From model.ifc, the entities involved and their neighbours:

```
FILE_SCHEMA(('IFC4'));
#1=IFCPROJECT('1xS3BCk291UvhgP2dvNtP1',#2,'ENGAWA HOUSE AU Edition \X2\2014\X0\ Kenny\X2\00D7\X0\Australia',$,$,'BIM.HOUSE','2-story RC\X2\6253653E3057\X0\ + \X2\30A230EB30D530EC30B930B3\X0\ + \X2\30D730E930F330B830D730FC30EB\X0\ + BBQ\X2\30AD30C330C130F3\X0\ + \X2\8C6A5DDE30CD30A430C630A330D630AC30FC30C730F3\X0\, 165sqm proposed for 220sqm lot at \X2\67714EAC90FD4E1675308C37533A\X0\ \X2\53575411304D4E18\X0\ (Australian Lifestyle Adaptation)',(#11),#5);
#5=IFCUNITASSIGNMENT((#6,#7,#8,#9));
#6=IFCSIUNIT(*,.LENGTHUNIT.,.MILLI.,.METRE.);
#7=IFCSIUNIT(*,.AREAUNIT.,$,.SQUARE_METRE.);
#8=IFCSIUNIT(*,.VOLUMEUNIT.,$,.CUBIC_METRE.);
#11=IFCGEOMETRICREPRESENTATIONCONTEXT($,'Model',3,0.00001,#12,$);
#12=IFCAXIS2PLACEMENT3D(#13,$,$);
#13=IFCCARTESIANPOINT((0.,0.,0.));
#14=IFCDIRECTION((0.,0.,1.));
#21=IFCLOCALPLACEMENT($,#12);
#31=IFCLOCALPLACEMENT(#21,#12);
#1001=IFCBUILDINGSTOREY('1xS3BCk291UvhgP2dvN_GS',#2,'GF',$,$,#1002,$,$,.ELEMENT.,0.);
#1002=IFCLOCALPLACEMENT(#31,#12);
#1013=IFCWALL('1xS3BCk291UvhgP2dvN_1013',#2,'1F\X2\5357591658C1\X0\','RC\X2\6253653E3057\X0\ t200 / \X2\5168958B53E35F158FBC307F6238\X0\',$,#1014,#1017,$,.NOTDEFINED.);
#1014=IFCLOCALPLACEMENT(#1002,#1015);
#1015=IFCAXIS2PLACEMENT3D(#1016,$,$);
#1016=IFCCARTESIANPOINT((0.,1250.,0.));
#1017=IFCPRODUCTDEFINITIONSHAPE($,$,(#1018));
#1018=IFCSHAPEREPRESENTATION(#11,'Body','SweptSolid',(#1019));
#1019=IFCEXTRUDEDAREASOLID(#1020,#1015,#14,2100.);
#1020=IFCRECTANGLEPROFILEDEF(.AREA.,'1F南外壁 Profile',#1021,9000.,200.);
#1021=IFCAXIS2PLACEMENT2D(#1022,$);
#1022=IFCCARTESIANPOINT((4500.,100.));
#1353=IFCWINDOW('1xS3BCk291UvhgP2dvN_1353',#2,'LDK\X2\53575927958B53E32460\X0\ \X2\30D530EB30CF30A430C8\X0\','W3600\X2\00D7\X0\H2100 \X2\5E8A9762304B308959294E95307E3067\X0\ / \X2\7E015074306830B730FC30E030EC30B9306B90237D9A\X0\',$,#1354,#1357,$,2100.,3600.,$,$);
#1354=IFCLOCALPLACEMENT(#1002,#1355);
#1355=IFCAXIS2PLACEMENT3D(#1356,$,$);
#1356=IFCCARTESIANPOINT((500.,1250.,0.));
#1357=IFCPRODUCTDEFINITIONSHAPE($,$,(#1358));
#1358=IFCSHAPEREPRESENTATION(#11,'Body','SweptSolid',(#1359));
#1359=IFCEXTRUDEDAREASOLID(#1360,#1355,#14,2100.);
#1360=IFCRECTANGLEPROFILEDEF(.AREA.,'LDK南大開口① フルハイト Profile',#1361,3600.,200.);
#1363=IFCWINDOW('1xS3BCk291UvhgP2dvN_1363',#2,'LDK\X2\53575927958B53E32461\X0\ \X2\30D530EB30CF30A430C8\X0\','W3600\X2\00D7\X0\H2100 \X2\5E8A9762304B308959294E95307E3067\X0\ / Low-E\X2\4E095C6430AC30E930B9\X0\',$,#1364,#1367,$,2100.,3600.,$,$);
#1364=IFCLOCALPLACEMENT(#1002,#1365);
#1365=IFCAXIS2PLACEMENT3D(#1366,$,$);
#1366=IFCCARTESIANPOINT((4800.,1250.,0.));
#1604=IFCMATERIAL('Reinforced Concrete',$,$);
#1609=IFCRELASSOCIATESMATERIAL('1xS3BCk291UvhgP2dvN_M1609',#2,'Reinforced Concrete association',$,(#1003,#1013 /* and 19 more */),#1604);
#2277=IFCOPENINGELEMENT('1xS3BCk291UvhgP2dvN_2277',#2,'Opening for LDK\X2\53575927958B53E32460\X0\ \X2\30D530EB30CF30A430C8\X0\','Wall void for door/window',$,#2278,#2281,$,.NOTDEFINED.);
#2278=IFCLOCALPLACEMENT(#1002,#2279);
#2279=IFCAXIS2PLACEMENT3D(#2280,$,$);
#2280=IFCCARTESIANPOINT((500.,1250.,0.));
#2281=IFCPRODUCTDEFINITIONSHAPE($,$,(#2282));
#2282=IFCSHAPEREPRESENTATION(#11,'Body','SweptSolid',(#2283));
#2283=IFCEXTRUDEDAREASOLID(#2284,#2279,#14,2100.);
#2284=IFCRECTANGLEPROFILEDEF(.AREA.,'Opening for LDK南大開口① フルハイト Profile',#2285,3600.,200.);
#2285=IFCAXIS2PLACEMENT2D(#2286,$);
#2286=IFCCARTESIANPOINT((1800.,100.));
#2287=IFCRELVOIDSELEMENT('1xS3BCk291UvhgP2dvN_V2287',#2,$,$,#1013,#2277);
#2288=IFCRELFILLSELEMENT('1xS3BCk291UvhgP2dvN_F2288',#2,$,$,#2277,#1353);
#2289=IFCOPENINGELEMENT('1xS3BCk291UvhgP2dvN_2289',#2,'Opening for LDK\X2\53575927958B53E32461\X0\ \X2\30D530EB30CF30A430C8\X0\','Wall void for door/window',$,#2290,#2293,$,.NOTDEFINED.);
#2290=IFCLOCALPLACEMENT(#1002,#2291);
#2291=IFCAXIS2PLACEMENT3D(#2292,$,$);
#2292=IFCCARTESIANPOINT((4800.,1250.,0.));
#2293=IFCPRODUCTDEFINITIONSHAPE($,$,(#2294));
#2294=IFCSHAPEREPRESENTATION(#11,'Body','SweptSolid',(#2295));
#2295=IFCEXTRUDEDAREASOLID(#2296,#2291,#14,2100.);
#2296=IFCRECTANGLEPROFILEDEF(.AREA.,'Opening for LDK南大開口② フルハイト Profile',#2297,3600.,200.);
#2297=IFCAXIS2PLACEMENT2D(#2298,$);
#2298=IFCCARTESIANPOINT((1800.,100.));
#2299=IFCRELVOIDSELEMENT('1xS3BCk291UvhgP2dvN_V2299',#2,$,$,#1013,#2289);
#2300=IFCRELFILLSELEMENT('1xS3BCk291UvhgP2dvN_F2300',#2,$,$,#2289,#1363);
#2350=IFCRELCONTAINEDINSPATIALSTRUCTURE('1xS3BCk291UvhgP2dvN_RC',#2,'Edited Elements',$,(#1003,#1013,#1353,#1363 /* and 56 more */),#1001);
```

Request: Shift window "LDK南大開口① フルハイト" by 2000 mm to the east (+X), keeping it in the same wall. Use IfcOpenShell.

```python
import ifcopenshell
import ifcopenshell.api.geometry
import ifcopenshell.util.placement
import ifcopenshell.util.unit

model = ifcopenshell.open("model.ifc")
unit_scale = ifcopenshell.util.unit.calculate_unit_scale(model)

window = model.by_id(1353)
opening = window.FillsVoids[0].RelatingOpeningElement
wall = opening.VoidsElements[0].RelatingBuildingElement

wall_matrix = ifcopenshell.util.placement.get_local_placement(wall.ObjectPlacement)
shift = wall_matrix[:3, 0] * 2 / unit_scale
before = ifcopenshell.util.placement.get_local_placement(window.ObjectPlacement)[:3, 3].copy()

# The window is not placed relative to its opening, so move both.
for product in (opening, window):
    matrix = ifcopenshell.util.placement.get_local_placement(product.ObjectPlacement)
    matrix[:3, 3] += shift
    ifcopenshell.api.geometry.edit_object_placement(model, product=product, matrix=matrix, is_si=False)

after = ifcopenshell.util.placement.get_local_placement(window.ObjectPlacement)[:3, 3]
print("window moved by", (after - before).round(3) + 0.0)

model.write("model-out.ifc")
```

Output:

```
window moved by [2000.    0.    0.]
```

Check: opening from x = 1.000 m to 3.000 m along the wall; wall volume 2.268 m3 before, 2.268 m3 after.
